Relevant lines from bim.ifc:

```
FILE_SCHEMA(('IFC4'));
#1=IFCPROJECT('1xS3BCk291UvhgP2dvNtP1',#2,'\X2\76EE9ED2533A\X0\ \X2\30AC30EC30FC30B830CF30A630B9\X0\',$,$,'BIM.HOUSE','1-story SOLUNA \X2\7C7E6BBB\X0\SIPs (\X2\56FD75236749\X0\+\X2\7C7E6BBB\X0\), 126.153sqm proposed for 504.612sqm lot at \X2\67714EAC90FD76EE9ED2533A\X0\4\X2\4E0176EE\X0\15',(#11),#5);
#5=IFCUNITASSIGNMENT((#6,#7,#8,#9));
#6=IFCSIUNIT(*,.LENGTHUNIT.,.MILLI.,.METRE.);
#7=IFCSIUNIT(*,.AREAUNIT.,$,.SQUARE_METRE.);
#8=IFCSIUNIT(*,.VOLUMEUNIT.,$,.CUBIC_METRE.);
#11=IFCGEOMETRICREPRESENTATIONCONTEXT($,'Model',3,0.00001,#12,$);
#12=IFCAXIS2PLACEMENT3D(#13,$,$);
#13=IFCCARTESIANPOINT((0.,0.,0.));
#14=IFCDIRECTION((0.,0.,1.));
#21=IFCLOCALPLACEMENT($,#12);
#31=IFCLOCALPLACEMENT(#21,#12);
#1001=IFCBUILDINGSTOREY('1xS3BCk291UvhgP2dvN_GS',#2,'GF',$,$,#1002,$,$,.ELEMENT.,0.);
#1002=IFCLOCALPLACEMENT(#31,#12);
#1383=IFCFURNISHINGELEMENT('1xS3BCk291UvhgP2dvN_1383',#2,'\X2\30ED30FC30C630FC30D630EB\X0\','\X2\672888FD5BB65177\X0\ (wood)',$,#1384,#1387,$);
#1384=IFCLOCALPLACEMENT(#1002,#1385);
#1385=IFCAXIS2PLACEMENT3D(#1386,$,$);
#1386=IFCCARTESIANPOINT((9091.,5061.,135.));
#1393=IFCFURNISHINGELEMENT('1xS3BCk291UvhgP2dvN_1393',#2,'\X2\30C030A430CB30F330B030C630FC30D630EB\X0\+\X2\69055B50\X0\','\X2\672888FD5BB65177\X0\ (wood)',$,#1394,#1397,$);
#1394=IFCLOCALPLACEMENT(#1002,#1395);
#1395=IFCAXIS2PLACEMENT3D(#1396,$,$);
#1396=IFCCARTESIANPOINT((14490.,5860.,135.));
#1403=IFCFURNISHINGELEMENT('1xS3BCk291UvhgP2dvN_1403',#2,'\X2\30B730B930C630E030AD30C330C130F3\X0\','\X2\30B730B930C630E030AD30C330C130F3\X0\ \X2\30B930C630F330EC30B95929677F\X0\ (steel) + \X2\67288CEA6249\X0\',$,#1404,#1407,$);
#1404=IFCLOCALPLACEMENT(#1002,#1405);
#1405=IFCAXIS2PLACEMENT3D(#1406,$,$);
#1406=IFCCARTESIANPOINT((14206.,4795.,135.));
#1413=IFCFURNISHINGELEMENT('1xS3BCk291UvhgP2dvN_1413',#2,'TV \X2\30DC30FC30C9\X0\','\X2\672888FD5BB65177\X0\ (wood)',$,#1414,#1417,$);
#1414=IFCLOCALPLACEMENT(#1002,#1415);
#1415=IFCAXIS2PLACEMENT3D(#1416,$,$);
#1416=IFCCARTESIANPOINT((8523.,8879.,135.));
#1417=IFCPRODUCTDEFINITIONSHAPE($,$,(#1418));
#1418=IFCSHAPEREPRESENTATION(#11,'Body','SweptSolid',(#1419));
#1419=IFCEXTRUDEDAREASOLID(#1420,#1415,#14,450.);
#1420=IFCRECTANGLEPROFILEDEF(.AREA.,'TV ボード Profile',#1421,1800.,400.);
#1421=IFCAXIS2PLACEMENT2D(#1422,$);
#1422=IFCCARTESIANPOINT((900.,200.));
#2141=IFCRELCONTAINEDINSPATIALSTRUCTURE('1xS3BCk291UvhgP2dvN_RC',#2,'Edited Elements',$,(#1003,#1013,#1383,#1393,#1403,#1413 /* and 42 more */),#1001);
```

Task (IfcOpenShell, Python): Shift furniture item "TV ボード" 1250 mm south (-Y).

```python
import ifcopenshell
import ifcopenshell.api.geometry
import ifcopenshell.util.placement
import ifcopenshell.util.unit

model = ifcopenshell.open("bim.ifc")
unit_scale = ifcopenshell.util.unit.calculate_unit_scale(model)

item = model.by_id(1413)
matrix = ifcopenshell.util.placement.get_local_placement(item.ObjectPlacement)
matrix[1, 3] -= 1.25 / unit_scale
ifcopenshell.api.geometry.edit_object_placement(model, product=item, matrix=matrix, is_si=False)

print(ifcopenshell.util.placement.get_local_placement(item.ObjectPlacement).round(3) + 0.0)

model.write("bim_edited.ifc")
```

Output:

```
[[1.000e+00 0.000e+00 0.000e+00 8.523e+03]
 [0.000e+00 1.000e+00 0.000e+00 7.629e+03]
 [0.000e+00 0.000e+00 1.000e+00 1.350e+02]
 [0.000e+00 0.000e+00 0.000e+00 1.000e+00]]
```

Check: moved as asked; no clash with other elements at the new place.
